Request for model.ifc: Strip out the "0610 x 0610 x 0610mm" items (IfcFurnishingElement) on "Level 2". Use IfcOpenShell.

First a look at what the model holds.

```python
import ifcopenshell
import ifcopenshell.util.element

model = ifcopenshell.open("model.ifc")
print(model.schema)
storey = next(s for s in model.by_type("IfcBuildingStorey") if s.Name == "Level 2")
furniture = [e for e in ifcopenshell.util.element.get_decomposition(storey) if e.is_a("IfcFurnishingElement")]
seen = {}
for e in furniture:
    element_type = ifcopenshell.util.element.get_type(e)
    name = element_type.Name if element_type not in (None, e) else None
    seen[name] = seen.get(name, 0) + 1
for name, count in sorted(seen.items(), key=str):
    print(count, "x", name)
```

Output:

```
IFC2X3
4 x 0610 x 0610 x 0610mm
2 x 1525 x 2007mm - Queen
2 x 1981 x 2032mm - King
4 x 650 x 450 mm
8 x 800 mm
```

```python
import ifcopenshell
import ifcopenshell.api.root
import ifcopenshell.util.element

model = ifcopenshell.open("model.ifc")

storey = next(s for s in model.by_type("IfcBuildingStorey") if s.Name == "Level 2")
furniture = [e for e in ifcopenshell.util.element.get_decomposition(storey) if e.is_a("IfcFurnishingElement")]
targets = [e for e in furniture if (t := ifcopenshell.util.element.get_type(e)) not in (None, e) and t.Name == "0610 x 0610 x 0610mm"]

for e in targets:
    ifcopenshell.api.root.remove_product(model, product=e)
print(len(targets), "removed")

model.write("model_rev.ifc")
```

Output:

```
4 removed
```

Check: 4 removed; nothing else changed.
